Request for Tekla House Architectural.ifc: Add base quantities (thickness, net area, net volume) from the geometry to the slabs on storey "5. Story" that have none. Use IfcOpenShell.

First a look at what the model holds.

```python
import ifcopenshell
import ifcopenshell.util.element
import ifcopenshell.util.unit

model = ifcopenshell.open("Tekla House Architectural.ifc")
print(model.schema)
for unit_type in ("LENGTHUNIT", "AREAUNIT", "VOLUMEUNIT"):
    print(unit_type, ifcopenshell.util.unit.calculate_unit_scale(model, unit_type))
storey = next(s for s in model.by_type("IfcBuildingStorey") if s.Name == "5. Story")
slabs = [e for e in ifcopenshell.util.element.get_decomposition(storey) if e.is_a("IfcSlab")]
for e in sorted(slabs, key=lambda e: e.id()):
    print(e.id(), e.is_a(), e.Name, list(ifcopenshell.util.element.get_psets(e, qtos_only=True)), sep=" | ")
```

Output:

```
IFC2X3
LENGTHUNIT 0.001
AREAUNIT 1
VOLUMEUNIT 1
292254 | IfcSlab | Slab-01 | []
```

```python
import ifcopenshell
import ifcopenshell.api.pset
import ifcopenshell.geom
import ifcopenshell.util.element
import ifcopenshell.util.shape
import ifcopenshell.util.unit

model = ifcopenshell.open("Tekla House Architectural.ifc")
unit_scale = ifcopenshell.util.unit.calculate_unit_scale(model)
area_scale = ifcopenshell.util.unit.calculate_unit_scale(model, "AREAUNIT")
volume_scale = ifcopenshell.util.unit.calculate_unit_scale(model, "VOLUMEUNIT")
settings = ifcopenshell.geom.settings()

storey = next(s for s in model.by_type("IfcBuildingStorey") if s.Name == "5. Story")
slabs = [e for e in ifcopenshell.util.element.get_decomposition(storey) if e.is_a("IfcSlab")]

for e in sorted(slabs, key=lambda e: e.id()):
    if ifcopenshell.util.element.get_psets(e, qtos_only=True, should_inherit=False):
        continue
    # Geometry comes back in metres, in the element's own axes.
    shape = ifcopenshell.geom.create_shape(settings, e)
    values = {
        "Width": ifcopenshell.util.shape.get_z(shape.geometry) / unit_scale,
        "NetArea": ifcopenshell.util.shape.get_footprint_area(shape.geometry) / area_scale,
        "NetVolume": ifcopenshell.util.shape.get_volume(shape.geometry) / volume_scale,
    }
    qto = ifcopenshell.api.pset.add_qto(model, product=e, name="BaseQuantities")
    ifcopenshell.api.pset.edit_qto(model, qto=qto, properties=values)
    print(e.id(), {k: round(v, 3) for k, v in values.items()})

model.write("Tekla House Architectural_updated.ifc")
```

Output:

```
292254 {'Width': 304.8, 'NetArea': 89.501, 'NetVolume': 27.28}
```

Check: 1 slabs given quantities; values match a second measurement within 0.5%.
